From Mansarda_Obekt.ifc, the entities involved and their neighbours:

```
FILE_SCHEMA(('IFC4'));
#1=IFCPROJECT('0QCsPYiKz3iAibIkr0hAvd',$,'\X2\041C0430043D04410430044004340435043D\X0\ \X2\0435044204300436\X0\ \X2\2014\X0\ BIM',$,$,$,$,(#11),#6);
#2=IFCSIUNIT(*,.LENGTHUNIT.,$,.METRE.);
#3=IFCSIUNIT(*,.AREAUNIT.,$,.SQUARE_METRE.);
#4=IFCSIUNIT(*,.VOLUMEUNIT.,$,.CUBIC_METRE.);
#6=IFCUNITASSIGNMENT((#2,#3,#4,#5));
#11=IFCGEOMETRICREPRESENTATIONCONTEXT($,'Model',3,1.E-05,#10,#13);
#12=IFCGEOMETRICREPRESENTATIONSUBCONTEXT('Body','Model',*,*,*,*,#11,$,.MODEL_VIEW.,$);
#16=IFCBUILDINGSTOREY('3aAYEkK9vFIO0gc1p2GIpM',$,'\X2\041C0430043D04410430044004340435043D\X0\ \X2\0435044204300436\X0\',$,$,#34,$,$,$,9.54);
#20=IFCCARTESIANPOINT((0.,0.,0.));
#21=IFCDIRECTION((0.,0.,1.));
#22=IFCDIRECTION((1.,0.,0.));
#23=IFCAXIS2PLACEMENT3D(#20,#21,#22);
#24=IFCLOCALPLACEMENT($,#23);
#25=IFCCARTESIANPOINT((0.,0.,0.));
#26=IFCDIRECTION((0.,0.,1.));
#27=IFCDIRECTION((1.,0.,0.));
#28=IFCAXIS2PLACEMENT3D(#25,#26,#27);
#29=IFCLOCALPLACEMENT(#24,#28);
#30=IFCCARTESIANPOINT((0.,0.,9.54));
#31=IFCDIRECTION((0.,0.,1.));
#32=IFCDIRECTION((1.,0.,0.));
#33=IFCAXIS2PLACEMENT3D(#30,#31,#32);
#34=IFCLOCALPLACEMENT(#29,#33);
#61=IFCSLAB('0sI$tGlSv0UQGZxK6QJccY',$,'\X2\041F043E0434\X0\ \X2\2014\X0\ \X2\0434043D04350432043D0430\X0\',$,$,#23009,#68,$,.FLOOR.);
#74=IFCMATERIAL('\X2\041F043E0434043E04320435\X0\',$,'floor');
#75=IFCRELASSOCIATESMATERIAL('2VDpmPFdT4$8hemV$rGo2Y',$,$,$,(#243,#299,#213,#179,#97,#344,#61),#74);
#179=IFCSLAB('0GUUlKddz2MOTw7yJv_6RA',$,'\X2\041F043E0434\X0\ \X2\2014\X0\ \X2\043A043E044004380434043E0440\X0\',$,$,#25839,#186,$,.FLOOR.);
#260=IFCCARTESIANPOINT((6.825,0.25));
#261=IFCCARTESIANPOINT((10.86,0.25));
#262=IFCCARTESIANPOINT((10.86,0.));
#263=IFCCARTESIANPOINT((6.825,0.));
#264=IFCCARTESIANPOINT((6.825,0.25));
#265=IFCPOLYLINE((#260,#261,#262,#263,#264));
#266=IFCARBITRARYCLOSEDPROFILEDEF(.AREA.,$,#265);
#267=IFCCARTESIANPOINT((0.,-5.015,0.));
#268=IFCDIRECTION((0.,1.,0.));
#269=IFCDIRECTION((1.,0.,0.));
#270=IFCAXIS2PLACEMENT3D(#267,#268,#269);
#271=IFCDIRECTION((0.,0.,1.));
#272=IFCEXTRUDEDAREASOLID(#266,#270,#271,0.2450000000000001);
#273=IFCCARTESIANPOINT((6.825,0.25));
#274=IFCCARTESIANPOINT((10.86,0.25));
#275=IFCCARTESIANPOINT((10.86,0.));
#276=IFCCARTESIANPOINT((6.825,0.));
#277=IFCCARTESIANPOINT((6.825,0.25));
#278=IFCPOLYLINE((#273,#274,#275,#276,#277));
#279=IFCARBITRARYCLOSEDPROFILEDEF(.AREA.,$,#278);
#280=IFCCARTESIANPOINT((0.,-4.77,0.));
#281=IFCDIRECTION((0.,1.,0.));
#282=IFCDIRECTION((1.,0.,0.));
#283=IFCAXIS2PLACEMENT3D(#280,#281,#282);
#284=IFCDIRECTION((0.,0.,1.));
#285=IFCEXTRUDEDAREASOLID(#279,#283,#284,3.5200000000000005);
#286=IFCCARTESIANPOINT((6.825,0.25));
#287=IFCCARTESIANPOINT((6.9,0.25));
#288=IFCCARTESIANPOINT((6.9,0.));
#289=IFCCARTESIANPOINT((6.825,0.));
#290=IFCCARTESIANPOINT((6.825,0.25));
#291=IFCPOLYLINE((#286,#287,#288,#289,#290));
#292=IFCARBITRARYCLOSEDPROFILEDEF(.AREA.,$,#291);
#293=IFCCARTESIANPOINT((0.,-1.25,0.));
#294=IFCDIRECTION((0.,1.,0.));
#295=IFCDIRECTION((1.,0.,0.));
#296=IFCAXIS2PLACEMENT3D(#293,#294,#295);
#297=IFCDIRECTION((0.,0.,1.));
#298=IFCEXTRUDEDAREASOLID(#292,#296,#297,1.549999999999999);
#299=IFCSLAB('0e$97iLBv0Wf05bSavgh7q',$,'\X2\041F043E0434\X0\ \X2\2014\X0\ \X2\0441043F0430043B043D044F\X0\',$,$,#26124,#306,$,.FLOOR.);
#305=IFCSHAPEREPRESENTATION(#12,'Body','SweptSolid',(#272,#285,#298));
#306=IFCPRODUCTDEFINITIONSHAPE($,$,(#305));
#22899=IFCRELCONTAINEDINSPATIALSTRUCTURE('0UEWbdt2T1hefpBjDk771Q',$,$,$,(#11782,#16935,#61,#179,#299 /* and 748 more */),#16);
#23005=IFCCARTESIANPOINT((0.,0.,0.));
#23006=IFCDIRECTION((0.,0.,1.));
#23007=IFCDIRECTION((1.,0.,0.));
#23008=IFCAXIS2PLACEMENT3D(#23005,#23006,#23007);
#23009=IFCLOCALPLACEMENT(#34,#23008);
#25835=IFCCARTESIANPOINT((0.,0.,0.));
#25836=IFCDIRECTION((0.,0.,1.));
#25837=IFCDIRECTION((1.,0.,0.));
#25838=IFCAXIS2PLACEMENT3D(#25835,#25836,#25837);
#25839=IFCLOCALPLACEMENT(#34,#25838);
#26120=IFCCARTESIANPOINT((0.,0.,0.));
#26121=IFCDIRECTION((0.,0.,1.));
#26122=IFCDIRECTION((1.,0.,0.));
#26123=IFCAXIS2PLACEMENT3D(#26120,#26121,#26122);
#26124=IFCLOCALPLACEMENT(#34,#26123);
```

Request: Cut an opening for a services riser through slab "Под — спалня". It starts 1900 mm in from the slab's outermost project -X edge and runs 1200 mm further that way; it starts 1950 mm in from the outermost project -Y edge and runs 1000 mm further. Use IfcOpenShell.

```python
import numpy as np
import ifcopenshell
import ifcopenshell.api.feature
import ifcopenshell.api.geometry
import ifcopenshell.api.root
import ifcopenshell.geom
import ifcopenshell.util.placement
import ifcopenshell.util.representation
import ifcopenshell.util.shape
import ifcopenshell.util.unit

model = ifcopenshell.open("Mansarda_Obekt.ifc")
unit_scale = ifcopenshell.util.unit.calculate_unit_scale(model)
settings = ifcopenshell.geom.settings()


def volume(element):
    """Net volume in cubic metres, openings subtracted."""
    shape = ifcopenshell.geom.create_shape(settings, element)
    return ifcopenshell.util.shape.get_volume(shape.geometry)


slab = model.by_id(299)
before = volume(slab)

# Extent in the slab's own axes, in metres. The edges named are its -X and -Y sides.
slab_shape = ifcopenshell.geom.create_shape(settings, slab)
vertices = ifcopenshell.util.shape.get_vertices(slab_shape.geometry)
x_min, y_min, bottom = vertices.min(axis=0)
top = vertices[:, 2].max()

opening = ifcopenshell.api.root.create_entity(model, ifc_class="IfcOpeningElement", name="Services riser opening", predefined_type="OPENING")
context = ifcopenshell.util.representation.get_context(model, "Model", "Body", "MODEL_VIEW")
width, depth = 1.2, 1
outline = [(0.0, 0.0), (width, 0.0), (width, depth), (0.0, depth), (0.0, 0.0)]
# Overshoot both faces by 50 mm so the cut is clean.
shape = ifcopenshell.api.geometry.add_slab_representation(
    model, context=context, depth=top - bottom + 0.1, polyline=outline
)
ifcopenshell.api.geometry.assign_representation(model, product=opening, representation=shape)

matrix = ifcopenshell.util.placement.get_local_placement(slab.ObjectPlacement)
matrix[:, 3] = matrix @ np.append(np.array([x_min + 1.9, y_min + 1.95, bottom - 0.05]) / unit_scale, 1.0)
ifcopenshell.api.geometry.edit_object_placement(model, product=opening, matrix=matrix, is_si=False)
ifcopenshell.api.feature.add_feature(model, feature=opening, element=slab)

after = volume(slab)

print(f"slab volume {before:.3f} -> {after:.3f} m3")

model.write("Mansarda_Obekt-out.ifc")
```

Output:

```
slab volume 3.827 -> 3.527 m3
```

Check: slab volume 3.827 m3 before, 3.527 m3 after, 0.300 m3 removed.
